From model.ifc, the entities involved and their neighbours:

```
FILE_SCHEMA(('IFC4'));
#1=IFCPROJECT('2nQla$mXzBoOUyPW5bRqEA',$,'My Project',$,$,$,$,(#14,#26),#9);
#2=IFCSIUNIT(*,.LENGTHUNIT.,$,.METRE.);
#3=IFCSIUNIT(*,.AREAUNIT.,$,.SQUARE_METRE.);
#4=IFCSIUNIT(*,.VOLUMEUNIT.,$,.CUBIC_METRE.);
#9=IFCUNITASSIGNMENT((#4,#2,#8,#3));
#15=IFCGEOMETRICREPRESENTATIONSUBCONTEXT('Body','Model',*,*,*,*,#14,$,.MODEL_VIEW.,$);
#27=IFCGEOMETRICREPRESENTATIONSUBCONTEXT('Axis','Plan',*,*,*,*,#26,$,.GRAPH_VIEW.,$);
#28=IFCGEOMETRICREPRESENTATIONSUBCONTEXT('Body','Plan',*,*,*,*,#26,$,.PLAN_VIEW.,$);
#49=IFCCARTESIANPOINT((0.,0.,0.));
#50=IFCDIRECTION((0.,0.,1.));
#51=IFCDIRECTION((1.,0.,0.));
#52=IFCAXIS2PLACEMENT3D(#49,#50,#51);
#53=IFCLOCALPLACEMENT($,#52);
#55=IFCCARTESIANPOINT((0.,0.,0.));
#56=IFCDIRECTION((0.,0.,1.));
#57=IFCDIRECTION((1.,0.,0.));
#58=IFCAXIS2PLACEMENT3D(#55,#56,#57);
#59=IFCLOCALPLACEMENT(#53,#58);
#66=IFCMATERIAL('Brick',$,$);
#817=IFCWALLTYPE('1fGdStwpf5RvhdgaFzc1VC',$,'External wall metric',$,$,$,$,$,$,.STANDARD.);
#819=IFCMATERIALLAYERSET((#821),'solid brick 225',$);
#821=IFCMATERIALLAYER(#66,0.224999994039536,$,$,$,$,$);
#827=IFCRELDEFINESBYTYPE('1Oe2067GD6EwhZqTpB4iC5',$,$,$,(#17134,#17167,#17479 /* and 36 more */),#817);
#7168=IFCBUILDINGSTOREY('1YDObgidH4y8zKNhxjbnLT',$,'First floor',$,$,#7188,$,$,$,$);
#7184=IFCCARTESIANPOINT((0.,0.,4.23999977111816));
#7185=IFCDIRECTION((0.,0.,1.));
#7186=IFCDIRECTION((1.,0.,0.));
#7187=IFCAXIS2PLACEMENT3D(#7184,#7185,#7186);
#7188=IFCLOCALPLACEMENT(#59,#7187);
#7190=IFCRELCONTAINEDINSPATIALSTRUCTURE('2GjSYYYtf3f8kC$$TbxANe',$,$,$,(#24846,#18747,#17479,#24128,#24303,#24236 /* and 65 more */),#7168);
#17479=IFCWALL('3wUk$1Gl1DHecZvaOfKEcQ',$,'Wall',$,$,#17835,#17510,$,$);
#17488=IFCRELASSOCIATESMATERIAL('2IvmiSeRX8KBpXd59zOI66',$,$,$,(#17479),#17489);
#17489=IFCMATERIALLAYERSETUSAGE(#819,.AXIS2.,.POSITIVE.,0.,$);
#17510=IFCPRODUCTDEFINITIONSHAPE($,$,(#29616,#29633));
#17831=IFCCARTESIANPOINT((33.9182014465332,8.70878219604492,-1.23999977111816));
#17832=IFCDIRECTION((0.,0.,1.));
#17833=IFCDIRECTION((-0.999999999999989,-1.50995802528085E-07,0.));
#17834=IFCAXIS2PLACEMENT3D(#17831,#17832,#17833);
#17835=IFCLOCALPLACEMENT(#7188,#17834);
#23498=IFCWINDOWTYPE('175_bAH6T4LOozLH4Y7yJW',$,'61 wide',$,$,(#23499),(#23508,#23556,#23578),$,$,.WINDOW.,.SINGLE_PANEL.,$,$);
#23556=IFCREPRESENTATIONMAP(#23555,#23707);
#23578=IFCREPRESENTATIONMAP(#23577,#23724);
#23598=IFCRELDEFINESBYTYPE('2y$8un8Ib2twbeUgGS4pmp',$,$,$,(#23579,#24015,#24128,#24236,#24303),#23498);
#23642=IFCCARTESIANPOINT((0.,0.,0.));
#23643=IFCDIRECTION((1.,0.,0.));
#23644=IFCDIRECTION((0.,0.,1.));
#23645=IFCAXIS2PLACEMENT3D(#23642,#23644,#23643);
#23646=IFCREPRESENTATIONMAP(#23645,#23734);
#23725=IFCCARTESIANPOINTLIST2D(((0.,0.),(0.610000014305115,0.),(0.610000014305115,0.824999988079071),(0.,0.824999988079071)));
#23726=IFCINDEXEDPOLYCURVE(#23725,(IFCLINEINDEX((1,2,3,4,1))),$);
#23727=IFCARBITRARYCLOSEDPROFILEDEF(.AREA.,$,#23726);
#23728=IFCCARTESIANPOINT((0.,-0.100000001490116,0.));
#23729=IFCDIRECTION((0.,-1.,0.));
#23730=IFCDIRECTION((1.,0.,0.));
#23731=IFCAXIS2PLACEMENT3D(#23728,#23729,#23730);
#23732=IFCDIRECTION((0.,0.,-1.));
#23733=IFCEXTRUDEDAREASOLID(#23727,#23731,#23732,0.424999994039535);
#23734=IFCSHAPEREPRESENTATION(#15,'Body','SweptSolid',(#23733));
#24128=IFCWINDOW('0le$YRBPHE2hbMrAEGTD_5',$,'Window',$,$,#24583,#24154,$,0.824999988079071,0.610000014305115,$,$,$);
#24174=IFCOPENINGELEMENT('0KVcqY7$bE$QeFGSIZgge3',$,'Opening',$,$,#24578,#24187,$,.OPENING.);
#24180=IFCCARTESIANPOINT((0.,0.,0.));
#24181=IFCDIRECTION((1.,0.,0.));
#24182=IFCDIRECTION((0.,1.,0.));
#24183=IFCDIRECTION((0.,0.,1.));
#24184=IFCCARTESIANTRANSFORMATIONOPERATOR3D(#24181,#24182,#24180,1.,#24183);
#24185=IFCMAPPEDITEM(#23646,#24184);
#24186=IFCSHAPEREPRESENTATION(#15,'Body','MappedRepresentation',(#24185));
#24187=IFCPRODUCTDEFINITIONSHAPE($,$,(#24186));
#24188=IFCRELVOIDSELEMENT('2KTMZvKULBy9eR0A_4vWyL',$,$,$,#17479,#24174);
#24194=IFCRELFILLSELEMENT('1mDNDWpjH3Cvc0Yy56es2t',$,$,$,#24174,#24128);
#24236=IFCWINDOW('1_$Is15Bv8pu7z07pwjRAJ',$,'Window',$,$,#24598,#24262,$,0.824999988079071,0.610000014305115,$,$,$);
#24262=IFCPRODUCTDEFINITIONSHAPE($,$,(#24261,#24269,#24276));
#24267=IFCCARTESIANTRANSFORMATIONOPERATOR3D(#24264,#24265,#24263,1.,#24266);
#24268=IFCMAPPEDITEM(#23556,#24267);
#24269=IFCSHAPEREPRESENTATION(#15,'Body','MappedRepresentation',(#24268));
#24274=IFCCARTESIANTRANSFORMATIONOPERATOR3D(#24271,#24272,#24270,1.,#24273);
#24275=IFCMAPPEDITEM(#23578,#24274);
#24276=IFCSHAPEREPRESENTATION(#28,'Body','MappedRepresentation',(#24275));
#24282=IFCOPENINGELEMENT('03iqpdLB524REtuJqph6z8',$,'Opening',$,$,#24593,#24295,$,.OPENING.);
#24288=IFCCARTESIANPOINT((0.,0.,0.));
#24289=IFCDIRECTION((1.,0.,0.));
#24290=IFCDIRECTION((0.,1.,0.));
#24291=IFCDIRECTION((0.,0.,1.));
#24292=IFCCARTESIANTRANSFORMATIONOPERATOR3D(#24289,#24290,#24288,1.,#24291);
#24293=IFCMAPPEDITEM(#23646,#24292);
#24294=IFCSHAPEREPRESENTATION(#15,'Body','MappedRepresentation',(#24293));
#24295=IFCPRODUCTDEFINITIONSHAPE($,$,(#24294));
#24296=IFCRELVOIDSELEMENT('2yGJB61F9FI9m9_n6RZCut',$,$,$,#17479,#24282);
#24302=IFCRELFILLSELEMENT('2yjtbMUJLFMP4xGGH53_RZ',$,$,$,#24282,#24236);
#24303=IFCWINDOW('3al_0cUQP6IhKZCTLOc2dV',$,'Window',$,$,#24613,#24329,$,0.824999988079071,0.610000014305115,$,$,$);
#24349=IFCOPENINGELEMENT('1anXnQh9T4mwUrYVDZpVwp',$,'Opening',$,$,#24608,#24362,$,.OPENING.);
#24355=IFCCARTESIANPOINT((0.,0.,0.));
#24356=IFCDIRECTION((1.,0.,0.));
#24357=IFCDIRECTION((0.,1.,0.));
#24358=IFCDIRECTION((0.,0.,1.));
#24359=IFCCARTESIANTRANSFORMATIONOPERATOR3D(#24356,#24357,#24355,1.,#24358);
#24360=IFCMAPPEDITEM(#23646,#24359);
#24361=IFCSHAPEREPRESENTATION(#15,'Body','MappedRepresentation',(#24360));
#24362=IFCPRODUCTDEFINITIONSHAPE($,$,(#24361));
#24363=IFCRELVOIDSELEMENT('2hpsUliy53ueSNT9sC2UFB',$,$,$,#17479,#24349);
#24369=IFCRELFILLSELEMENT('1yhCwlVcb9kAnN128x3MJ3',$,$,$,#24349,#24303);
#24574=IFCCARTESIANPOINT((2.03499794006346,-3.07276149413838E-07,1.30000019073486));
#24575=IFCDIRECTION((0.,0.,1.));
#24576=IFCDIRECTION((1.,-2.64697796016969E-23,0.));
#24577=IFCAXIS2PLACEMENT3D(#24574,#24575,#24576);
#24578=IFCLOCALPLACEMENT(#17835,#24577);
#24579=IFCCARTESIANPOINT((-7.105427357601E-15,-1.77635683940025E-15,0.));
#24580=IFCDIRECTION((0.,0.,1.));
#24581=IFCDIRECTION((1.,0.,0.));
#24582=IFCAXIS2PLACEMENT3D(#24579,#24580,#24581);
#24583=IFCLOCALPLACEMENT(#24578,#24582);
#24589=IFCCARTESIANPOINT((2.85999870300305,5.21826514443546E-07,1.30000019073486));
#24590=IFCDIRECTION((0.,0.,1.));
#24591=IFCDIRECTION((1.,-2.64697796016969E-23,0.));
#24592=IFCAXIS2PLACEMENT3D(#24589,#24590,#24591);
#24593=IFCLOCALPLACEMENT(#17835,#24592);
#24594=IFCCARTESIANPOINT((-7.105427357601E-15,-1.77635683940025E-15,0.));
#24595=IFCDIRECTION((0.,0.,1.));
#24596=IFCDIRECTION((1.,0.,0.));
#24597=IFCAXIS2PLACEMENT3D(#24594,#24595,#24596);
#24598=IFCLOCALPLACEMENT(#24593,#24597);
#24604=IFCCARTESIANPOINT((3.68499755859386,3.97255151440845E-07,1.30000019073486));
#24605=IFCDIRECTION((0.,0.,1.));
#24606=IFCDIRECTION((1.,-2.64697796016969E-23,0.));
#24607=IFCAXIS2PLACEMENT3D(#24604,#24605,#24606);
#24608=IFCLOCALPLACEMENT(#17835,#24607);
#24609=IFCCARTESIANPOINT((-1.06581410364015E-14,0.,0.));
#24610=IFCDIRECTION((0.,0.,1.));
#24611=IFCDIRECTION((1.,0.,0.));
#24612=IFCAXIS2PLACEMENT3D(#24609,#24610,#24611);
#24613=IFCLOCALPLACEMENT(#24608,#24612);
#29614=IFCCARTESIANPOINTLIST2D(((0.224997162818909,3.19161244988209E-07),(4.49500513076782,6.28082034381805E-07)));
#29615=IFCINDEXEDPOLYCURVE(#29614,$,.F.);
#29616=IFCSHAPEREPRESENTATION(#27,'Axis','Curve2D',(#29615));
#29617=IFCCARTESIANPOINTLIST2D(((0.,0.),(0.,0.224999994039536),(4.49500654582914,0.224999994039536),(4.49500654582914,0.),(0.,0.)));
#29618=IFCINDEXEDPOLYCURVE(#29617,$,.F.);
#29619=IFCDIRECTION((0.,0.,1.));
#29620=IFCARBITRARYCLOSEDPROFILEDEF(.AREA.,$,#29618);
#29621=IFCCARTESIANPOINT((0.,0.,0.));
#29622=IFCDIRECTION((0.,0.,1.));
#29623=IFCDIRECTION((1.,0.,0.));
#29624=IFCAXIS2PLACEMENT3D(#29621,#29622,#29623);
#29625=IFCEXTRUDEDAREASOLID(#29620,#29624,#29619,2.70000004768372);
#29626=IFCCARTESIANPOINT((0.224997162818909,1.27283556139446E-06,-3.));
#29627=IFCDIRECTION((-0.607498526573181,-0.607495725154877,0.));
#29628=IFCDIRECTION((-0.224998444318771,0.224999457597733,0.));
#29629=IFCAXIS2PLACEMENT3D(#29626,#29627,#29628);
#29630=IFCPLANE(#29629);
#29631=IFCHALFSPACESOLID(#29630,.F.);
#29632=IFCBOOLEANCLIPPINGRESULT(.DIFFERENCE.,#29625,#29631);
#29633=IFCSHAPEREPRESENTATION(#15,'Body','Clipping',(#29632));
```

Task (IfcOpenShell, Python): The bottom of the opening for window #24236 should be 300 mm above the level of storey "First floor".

```python
import numpy as np
import ifcopenshell
import ifcopenshell.api.geometry
import ifcopenshell.geom
import ifcopenshell.util.element
import ifcopenshell.util.placement
import ifcopenshell.util.shape
import ifcopenshell.util.unit

model = ifcopenshell.open("model.ifc")
unit_scale = ifcopenshell.util.unit.calculate_unit_scale(model)

window = model.by_guid("1_$Is15Bv8pu7z07pwjRAJ")
opening = window.FillsVoids[0].RelatingOpeningElement
storey = ifcopenshell.util.element.get_container(window, ifc_class="IfcBuildingStorey")
level = ifcopenshell.util.placement.get_local_placement(storey.ObjectPlacement)[2, 3]

# The opening's origin need not be at the sill, so measure its lowest point.
shape = ifcopenshell.geom.create_shape(ifcopenshell.geom.settings(), opening)
bottom = ifcopenshell.util.shape.get_shape_bottom_elevation(shape, shape.geometry) / unit_scale
dz = level + 0.3 - bottom

shift = np.array([0.0, 0.0, dz])
# The window is placed relative to its opening, so it follows when the opening moves.
matrix = ifcopenshell.util.placement.get_local_placement(opening.ObjectPlacement)
matrix[:3, 3] += shift
ifcopenshell.api.geometry.edit_object_placement(
    model, product=opening, matrix=matrix, is_si=False, should_transform_children=True
)

print(f"moved by {dz * unit_scale:+.3f} m")

model.write("model_rev.ifc")
```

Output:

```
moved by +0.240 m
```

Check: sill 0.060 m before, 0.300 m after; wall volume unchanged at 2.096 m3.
